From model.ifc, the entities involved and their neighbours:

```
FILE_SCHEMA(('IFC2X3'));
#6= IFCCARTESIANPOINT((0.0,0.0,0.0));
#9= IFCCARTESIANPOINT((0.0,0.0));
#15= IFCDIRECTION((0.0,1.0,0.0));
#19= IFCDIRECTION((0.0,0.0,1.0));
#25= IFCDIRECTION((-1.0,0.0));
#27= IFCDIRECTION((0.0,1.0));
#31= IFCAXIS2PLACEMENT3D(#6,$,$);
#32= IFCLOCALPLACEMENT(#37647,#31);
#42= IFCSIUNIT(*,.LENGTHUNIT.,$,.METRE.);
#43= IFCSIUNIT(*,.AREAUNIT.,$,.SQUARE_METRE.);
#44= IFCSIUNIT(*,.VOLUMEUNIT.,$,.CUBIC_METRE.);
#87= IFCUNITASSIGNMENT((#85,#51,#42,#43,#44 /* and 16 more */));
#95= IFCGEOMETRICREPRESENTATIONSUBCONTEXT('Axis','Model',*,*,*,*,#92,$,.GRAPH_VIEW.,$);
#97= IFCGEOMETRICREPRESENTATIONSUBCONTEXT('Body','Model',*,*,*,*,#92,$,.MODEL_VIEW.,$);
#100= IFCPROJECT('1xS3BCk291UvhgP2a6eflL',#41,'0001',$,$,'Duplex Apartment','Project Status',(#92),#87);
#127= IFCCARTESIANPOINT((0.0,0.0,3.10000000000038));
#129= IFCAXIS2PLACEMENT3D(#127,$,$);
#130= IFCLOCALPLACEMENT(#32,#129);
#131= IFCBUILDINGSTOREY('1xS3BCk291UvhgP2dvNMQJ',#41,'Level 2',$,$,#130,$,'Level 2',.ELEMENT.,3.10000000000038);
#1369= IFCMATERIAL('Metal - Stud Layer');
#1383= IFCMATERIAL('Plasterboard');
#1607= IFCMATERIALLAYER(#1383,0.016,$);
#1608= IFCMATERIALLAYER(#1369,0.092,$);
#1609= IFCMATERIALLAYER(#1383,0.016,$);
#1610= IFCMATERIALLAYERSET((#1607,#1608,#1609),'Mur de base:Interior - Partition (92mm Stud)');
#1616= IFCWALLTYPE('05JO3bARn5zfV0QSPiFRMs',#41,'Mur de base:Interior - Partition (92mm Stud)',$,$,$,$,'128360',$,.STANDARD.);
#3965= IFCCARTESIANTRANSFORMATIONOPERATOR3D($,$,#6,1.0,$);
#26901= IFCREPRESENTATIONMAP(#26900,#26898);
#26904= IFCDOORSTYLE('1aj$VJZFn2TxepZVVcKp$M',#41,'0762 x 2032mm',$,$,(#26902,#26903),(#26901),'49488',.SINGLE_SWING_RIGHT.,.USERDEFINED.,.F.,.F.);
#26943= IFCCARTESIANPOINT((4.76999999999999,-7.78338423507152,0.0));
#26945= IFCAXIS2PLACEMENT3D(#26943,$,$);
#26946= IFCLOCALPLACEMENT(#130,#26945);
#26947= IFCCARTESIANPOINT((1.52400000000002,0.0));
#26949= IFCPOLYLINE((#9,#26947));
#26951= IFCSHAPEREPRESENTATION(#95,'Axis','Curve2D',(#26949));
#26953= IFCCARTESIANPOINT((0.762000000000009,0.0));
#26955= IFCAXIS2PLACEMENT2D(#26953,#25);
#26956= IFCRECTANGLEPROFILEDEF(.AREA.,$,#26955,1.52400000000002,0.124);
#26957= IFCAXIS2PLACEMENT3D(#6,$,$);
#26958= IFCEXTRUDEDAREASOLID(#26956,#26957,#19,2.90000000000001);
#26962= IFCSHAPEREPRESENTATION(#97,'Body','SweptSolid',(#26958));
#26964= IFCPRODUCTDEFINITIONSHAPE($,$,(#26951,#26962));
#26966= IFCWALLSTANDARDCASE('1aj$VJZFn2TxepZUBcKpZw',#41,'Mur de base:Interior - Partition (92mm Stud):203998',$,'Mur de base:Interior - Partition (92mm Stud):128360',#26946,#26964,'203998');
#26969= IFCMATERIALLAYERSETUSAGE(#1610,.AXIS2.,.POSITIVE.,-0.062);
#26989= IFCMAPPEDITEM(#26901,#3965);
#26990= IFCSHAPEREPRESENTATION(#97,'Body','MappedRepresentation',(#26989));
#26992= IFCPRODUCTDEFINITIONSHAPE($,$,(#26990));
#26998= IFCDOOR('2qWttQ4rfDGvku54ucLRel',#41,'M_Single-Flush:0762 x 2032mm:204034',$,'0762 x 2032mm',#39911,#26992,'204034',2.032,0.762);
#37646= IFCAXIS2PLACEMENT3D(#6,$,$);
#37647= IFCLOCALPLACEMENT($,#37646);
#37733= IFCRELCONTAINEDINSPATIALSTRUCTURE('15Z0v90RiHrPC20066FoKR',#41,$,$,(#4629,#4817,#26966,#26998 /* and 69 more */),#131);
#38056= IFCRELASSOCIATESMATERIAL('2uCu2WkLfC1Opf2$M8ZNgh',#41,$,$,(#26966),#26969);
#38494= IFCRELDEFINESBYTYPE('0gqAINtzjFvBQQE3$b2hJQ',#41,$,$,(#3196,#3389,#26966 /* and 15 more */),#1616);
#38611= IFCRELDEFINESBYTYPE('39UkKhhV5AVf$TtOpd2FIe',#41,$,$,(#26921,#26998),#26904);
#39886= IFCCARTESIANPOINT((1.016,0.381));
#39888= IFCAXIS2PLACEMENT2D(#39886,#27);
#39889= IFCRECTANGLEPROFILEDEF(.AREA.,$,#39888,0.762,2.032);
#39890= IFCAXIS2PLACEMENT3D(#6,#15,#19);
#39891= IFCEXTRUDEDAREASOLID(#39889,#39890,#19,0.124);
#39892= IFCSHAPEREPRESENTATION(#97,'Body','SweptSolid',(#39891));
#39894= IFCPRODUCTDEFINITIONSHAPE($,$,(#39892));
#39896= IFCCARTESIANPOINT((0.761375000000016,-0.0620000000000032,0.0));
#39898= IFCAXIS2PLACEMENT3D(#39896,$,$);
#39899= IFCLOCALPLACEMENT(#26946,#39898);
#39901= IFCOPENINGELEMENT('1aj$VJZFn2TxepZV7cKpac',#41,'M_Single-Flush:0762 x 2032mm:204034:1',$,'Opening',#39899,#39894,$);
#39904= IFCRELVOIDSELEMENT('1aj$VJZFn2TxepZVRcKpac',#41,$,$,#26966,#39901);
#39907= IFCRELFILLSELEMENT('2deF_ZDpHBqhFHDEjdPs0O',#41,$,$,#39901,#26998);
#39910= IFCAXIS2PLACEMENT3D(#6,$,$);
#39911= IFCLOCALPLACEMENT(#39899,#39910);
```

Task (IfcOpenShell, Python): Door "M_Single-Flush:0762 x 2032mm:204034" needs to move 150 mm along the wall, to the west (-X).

```python
import ifcopenshell
import ifcopenshell.api.geometry
import ifcopenshell.util.placement

model = ifcopenshell.open("model.ifc")

door = model.by_guid("2qWttQ4rfDGvku54ucLRel")
opening = door.FillsVoids[0].RelatingOpeningElement
wall = opening.VoidsElements[0].RelatingBuildingElement

wall_matrix = ifcopenshell.util.placement.get_local_placement(wall.ObjectPlacement)
shift = wall_matrix[:3, 0] * -0.15
before = ifcopenshell.util.placement.get_local_placement(door.ObjectPlacement)[:3, 3].copy()

# The door is placed relative to its opening, so it follows when the opening moves.
matrix = ifcopenshell.util.placement.get_local_placement(opening.ObjectPlacement)
matrix[:3, 3] += shift
ifcopenshell.api.geometry.edit_object_placement(
    model, product=opening, matrix=matrix, is_si=False, should_transform_children=True
)

after = ifcopenshell.util.placement.get_local_placement(door.ObjectPlacement)[:3, 3]
print("door moved by", (after - before).round(3) + 0.0)

model.write("model_rev.ifc")
```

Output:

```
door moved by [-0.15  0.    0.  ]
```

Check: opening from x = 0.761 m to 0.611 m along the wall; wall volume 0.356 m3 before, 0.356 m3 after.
